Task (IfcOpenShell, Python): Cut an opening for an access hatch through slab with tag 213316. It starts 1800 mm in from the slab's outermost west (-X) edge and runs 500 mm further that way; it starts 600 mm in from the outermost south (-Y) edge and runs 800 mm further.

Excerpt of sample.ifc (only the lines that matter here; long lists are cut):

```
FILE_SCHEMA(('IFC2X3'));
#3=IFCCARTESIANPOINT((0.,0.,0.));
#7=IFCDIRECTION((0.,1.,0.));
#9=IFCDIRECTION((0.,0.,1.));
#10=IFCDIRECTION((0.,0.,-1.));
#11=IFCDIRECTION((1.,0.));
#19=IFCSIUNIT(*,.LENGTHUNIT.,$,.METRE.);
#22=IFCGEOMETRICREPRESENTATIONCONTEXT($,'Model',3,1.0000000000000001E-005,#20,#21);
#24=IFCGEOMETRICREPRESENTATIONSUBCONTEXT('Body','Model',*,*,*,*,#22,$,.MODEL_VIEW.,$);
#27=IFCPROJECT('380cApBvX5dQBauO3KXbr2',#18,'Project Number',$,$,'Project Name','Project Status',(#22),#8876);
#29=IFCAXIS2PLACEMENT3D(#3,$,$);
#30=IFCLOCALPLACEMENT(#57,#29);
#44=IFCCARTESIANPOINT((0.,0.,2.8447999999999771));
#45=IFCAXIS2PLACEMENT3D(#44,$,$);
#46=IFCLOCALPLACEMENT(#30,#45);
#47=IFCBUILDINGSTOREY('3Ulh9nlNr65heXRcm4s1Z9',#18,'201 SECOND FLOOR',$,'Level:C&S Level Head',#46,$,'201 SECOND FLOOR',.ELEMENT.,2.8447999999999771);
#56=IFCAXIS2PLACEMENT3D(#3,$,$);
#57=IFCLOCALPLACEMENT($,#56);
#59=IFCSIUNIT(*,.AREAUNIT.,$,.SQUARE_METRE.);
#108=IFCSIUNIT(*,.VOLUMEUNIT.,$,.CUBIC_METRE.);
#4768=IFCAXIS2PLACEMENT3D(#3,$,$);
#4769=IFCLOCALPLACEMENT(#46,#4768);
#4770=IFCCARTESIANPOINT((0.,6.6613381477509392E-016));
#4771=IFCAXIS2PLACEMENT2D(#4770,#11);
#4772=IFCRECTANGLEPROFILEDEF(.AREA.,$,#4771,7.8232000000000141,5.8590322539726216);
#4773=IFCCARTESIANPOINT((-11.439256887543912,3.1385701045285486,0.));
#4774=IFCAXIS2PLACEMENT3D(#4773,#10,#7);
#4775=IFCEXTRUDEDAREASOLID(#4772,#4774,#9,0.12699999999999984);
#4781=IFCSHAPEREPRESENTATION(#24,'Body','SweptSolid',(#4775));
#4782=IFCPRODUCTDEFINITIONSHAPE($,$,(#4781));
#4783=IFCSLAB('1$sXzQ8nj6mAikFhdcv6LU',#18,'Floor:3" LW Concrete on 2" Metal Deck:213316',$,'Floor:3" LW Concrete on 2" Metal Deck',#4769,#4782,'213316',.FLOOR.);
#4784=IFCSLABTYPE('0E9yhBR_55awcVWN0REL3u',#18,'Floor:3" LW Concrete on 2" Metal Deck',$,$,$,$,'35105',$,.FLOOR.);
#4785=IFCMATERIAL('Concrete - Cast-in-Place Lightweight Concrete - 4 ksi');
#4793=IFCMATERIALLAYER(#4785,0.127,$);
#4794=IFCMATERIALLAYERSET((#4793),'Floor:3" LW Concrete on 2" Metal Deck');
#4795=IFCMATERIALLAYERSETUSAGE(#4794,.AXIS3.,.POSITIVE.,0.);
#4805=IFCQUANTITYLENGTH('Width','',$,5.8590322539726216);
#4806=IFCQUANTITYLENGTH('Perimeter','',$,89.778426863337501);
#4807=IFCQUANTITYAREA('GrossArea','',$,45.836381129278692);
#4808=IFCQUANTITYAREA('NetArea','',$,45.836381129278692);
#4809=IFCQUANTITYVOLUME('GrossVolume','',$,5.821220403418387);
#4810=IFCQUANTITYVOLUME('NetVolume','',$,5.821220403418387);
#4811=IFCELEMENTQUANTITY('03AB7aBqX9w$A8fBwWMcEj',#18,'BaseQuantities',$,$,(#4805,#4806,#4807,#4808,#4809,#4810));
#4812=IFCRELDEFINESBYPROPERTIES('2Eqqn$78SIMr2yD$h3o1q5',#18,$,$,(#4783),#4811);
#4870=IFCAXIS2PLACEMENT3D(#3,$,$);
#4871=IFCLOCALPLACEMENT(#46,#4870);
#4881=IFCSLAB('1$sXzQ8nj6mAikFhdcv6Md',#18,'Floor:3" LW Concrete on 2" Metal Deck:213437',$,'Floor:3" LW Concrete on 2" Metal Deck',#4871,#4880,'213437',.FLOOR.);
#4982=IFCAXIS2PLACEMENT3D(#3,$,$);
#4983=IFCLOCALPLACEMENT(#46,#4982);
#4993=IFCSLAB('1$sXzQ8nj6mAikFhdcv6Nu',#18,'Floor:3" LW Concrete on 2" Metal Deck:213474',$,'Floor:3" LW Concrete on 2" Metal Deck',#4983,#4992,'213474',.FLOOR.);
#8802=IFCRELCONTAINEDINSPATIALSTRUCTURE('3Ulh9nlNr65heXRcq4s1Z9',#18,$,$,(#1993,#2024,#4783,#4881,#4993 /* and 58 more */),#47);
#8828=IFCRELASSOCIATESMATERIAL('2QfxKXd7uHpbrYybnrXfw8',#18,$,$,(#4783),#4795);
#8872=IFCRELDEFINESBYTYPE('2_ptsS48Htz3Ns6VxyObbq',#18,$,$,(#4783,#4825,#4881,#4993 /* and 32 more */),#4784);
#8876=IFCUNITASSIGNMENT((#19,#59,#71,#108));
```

```python
import numpy as np
import ifcopenshell
import ifcopenshell.api.feature
import ifcopenshell.api.geometry
import ifcopenshell.api.pset
import ifcopenshell.api.root
import ifcopenshell.geom
import ifcopenshell.util.element
import ifcopenshell.util.placement
import ifcopenshell.util.representation
import ifcopenshell.util.shape
import ifcopenshell.util.unit

model = ifcopenshell.open("sample.ifc")
unit_scale = ifcopenshell.util.unit.calculate_unit_scale(model)
area_scale = ifcopenshell.util.unit.calculate_unit_scale(model, "AREAUNIT")
volume_scale = ifcopenshell.util.unit.calculate_unit_scale(model, "VOLUMEUNIT")
settings = ifcopenshell.geom.settings()


def volume(element):
    """Net volume in cubic metres, openings subtracted."""
    shape = ifcopenshell.geom.create_shape(settings, element)
    return ifcopenshell.util.shape.get_volume(shape.geometry)


slab = model.by_id(4783)
before = volume(slab)

# Extent in the slab's own axes, in metres. The edges named are its -X and -Y sides.
slab_shape = ifcopenshell.geom.create_shape(settings, slab)
vertices = ifcopenshell.util.shape.get_vertices(slab_shape.geometry)
x_min, y_min, bottom = vertices.min(axis=0)
top = vertices[:, 2].max()

opening = ifcopenshell.api.root.create_entity(model, ifc_class="IfcOpeningElement", name="Access hatch opening")
context = ifcopenshell.util.representation.get_context(model, "Model", "Body", "MODEL_VIEW")
width, depth = 0.5, 0.8
outline = [(0.0, 0.0), (width, 0.0), (width, depth), (0.0, depth), (0.0, 0.0)]
# Overshoot both faces by 50 mm so the cut is clean.
shape = ifcopenshell.api.geometry.add_slab_representation(
    model, context=context, depth=top - bottom + 0.1, polyline=outline
)
ifcopenshell.api.geometry.assign_representation(model, product=opening, representation=shape)

matrix = ifcopenshell.util.placement.get_local_placement(slab.ObjectPlacement)
matrix[:, 3] = matrix @ np.append(np.array([x_min + 1.8, y_min + 0.6, bottom - 0.05]) / unit_scale, 1.0)
ifcopenshell.api.geometry.edit_object_placement(model, product=opening, matrix=matrix, is_si=False)
ifcopenshell.api.feature.add_feature(model, feature=opening, element=slab)

after = volume(slab)

# Update the slab's stored quantities.
qto = model.by_id(ifcopenshell.util.element.get_pset(slab, "BaseQuantities", should_inherit=False)["id"])
ifcopenshell.api.pset.edit_qto(model, qto=qto, properties={
    "NetArea": after / (top - bottom) / area_scale,
    "NetVolume": after / volume_scale,
})

print(f"slab volume {before:.3f} -> {after:.3f} m3")

model.write("sample_edited.ifc")
```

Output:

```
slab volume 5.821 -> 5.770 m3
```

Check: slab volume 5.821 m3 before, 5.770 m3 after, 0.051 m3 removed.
